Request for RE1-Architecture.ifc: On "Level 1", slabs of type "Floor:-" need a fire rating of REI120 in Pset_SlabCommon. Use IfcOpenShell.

First a look at what the model holds.

```python
import ifcopenshell
import ifcopenshell.util.element

model = ifcopenshell.open("RE1-Architecture.ifc")
print(model.schema)
storey = next(s for s in model.by_type("IfcBuildingStorey") if s.Name == "Level 1")
slabs = [e for e in ifcopenshell.util.element.get_decomposition(storey) if e.is_a("IfcSlab")]
seen = {}
for e in slabs:
    element_type = ifcopenshell.util.element.get_type(e)
    key = (element_type.Name if element_type != e and element_type else None, ifcopenshell.util.element.get_pset(e, "Pset_SlabCommon", "FireRating"))
    seen[key] = seen.get(key, 0) + 1
for (name, value), count in sorted(seen.items(), key=str):
    print(count, "x", name, "|", value)
```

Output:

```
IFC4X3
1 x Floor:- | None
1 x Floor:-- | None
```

```python
import ifcopenshell
import ifcopenshell.api.pset
import ifcopenshell.util.element

model = ifcopenshell.open("RE1-Architecture.ifc")

storey = next(s for s in model.by_type("IfcBuildingStorey") if s.Name == "Level 1")
slabs = [e for e in ifcopenshell.util.element.get_decomposition(storey) if e.is_a("IfcSlab")]

count = 0
for e in slabs:
    element_type = ifcopenshell.util.element.get_type(e)
    if element_type in (None, e) or element_type.Name != "Floor:-":
        continue
    # add_pset returns the element's existing set when there is one.
    pset = ifcopenshell.api.pset.add_pset(model, product=e, name="Pset_SlabCommon")
    ifcopenshell.api.pset.edit_pset(model, pset=pset, properties={"FireRating": "REI120"})
    count += 1

print(count, "slabs updated")

model.write("RE1-Architecture_edited.ifc")
```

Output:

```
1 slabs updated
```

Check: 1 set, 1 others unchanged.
